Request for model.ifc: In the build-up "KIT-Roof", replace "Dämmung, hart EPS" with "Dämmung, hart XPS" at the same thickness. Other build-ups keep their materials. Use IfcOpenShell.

First a look at what the model holds.

```python
import ifcopenshell
import ifcopenshell.util.element

model = ifcopenshell.open("model.ifc")
print(model.schema)
for layer_set in model.by_type("IfcMaterialLayerSet"):
    if layer_set.LayerSetName == "KIT-Roof":
        for layer in layer_set.MaterialLayers:
            print(layer.id(), layer.Material and layer.Material.Name, layer.LayerThickness, sep=" | ")
        print(len(ifcopenshell.util.element.get_elements_by_material(model, layer_set)), "elements and types use it")
print(sorted(m.Name for m in model.by_type("IfcMaterial") if m.Name)[:60])
```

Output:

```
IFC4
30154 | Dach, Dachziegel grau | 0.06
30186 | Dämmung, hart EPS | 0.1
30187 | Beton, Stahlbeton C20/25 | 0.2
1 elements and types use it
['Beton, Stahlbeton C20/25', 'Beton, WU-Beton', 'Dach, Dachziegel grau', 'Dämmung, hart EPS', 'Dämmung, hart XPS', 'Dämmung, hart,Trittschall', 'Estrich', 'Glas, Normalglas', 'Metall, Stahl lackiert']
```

```python
import ifcopenshell
import ifcopenshell.api.material

model = ifcopenshell.open("model.ifc")

layer_set = next(s for s in model.by_type("IfcMaterialLayerSet") if s.LayerSetName == "KIT-Roof")
layer = next(l for l in layer_set.MaterialLayers if l.Material and l.Material.Name == "Dämmung, hart EPS")
material = next(m for m in model.by_type("IfcMaterial") if m.Name == "Dämmung, hart XPS")

# Point this one layer at the other material; renaming the old one would change it everywhere.
ifcopenshell.api.material.edit_layer(model, layer=layer, attributes={}, material=material)

print([l.Material.Name if l.Material else None for l in layer_set.MaterialLayers])

model.write("model_v2.ifc")
```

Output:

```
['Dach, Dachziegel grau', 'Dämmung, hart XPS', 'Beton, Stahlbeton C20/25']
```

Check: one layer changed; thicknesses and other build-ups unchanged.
